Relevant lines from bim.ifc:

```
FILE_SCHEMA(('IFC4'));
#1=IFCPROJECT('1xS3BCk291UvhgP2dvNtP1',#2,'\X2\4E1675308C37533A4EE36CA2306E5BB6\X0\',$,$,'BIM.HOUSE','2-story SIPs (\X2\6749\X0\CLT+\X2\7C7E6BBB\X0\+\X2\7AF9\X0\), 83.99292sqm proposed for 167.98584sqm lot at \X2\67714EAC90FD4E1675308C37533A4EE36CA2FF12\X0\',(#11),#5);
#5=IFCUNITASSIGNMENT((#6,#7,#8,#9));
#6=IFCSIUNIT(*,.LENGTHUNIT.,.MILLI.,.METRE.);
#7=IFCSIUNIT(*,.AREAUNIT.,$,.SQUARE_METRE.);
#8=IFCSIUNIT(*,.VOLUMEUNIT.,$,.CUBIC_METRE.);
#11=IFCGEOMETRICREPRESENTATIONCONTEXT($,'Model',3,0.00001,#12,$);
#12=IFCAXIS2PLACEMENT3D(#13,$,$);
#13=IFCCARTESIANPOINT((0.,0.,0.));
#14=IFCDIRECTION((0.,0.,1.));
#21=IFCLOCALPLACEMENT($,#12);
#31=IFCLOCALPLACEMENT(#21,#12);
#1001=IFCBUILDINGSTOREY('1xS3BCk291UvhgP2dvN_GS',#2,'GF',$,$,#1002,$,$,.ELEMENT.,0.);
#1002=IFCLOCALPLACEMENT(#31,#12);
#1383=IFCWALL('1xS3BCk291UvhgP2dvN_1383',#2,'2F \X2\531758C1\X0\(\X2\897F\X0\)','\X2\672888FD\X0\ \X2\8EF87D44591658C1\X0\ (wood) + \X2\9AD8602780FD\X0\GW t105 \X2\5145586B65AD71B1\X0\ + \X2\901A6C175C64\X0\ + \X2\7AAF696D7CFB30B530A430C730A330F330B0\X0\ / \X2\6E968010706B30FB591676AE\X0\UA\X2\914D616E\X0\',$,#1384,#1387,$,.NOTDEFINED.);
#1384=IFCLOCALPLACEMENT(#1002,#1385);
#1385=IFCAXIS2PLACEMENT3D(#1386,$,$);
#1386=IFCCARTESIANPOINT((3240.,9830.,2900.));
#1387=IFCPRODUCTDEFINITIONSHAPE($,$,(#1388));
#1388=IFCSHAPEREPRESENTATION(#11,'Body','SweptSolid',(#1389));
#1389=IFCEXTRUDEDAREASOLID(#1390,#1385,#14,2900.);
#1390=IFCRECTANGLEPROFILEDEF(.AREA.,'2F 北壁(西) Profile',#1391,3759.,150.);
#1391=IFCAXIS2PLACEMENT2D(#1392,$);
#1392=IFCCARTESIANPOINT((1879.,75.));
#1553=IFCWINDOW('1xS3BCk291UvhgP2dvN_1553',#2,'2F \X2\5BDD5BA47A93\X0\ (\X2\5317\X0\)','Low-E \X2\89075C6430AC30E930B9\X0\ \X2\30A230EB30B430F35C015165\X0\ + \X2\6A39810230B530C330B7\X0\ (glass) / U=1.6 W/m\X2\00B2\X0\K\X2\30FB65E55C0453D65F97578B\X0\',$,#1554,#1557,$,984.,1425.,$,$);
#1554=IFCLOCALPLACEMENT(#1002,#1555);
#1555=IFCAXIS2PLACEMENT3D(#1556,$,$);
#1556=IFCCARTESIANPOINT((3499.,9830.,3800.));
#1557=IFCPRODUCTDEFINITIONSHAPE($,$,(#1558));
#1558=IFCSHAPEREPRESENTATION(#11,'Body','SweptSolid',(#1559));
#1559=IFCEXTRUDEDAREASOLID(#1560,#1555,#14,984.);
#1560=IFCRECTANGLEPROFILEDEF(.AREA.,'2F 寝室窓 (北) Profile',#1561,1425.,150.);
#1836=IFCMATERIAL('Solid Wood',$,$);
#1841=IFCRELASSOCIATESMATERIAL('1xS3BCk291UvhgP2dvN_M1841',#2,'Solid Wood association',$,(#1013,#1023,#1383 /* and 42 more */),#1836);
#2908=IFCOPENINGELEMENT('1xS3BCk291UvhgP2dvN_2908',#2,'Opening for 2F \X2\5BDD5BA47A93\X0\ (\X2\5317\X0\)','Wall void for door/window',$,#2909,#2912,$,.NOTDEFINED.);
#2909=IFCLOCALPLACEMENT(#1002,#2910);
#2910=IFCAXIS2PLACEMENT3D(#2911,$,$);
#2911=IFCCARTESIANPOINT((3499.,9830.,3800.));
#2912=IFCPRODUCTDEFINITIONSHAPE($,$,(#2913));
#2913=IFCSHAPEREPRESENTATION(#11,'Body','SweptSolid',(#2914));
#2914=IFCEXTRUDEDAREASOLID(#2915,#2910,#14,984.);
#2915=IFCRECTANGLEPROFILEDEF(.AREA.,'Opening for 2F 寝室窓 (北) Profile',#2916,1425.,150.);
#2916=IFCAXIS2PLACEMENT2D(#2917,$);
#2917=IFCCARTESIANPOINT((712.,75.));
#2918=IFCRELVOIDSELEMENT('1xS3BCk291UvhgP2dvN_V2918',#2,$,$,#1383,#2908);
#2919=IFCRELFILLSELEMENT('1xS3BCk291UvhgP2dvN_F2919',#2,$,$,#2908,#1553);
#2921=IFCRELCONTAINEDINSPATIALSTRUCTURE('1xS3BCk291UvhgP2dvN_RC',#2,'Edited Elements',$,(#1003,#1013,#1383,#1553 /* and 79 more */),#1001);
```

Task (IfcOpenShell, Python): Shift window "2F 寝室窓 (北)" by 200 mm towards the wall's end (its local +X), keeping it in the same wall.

```python
import ifcopenshell
import ifcopenshell.api.geometry
import ifcopenshell.util.placement
import ifcopenshell.util.unit

model = ifcopenshell.open("bim.ifc")
unit_scale = ifcopenshell.util.unit.calculate_unit_scale(model)

window = model.by_guid("1xS3BCk291UvhgP2dvN_1553")
opening = window.FillsVoids[0].RelatingOpeningElement
wall = opening.VoidsElements[0].RelatingBuildingElement

wall_matrix = ifcopenshell.util.placement.get_local_placement(wall.ObjectPlacement)
shift = wall_matrix[:3, 0] * 0.2 / unit_scale
before = ifcopenshell.util.placement.get_local_placement(window.ObjectPlacement)[:3, 3].copy()

# The window is not placed relative to its opening, so move both.
for product in (opening, window):
    matrix = ifcopenshell.util.placement.get_local_placement(product.ObjectPlacement)
    matrix[:3, 3] += shift
    ifcopenshell.api.geometry.edit_object_placement(model, product=product, matrix=matrix, is_si=False)

after = ifcopenshell.util.placement.get_local_placement(window.ObjectPlacement)[:3, 3]
print("window moved by", (after - before).round(3) + 0.0)

model.write("bim-out.ifc")
```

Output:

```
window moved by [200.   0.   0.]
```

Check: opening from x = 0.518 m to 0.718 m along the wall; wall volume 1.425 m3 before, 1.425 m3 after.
